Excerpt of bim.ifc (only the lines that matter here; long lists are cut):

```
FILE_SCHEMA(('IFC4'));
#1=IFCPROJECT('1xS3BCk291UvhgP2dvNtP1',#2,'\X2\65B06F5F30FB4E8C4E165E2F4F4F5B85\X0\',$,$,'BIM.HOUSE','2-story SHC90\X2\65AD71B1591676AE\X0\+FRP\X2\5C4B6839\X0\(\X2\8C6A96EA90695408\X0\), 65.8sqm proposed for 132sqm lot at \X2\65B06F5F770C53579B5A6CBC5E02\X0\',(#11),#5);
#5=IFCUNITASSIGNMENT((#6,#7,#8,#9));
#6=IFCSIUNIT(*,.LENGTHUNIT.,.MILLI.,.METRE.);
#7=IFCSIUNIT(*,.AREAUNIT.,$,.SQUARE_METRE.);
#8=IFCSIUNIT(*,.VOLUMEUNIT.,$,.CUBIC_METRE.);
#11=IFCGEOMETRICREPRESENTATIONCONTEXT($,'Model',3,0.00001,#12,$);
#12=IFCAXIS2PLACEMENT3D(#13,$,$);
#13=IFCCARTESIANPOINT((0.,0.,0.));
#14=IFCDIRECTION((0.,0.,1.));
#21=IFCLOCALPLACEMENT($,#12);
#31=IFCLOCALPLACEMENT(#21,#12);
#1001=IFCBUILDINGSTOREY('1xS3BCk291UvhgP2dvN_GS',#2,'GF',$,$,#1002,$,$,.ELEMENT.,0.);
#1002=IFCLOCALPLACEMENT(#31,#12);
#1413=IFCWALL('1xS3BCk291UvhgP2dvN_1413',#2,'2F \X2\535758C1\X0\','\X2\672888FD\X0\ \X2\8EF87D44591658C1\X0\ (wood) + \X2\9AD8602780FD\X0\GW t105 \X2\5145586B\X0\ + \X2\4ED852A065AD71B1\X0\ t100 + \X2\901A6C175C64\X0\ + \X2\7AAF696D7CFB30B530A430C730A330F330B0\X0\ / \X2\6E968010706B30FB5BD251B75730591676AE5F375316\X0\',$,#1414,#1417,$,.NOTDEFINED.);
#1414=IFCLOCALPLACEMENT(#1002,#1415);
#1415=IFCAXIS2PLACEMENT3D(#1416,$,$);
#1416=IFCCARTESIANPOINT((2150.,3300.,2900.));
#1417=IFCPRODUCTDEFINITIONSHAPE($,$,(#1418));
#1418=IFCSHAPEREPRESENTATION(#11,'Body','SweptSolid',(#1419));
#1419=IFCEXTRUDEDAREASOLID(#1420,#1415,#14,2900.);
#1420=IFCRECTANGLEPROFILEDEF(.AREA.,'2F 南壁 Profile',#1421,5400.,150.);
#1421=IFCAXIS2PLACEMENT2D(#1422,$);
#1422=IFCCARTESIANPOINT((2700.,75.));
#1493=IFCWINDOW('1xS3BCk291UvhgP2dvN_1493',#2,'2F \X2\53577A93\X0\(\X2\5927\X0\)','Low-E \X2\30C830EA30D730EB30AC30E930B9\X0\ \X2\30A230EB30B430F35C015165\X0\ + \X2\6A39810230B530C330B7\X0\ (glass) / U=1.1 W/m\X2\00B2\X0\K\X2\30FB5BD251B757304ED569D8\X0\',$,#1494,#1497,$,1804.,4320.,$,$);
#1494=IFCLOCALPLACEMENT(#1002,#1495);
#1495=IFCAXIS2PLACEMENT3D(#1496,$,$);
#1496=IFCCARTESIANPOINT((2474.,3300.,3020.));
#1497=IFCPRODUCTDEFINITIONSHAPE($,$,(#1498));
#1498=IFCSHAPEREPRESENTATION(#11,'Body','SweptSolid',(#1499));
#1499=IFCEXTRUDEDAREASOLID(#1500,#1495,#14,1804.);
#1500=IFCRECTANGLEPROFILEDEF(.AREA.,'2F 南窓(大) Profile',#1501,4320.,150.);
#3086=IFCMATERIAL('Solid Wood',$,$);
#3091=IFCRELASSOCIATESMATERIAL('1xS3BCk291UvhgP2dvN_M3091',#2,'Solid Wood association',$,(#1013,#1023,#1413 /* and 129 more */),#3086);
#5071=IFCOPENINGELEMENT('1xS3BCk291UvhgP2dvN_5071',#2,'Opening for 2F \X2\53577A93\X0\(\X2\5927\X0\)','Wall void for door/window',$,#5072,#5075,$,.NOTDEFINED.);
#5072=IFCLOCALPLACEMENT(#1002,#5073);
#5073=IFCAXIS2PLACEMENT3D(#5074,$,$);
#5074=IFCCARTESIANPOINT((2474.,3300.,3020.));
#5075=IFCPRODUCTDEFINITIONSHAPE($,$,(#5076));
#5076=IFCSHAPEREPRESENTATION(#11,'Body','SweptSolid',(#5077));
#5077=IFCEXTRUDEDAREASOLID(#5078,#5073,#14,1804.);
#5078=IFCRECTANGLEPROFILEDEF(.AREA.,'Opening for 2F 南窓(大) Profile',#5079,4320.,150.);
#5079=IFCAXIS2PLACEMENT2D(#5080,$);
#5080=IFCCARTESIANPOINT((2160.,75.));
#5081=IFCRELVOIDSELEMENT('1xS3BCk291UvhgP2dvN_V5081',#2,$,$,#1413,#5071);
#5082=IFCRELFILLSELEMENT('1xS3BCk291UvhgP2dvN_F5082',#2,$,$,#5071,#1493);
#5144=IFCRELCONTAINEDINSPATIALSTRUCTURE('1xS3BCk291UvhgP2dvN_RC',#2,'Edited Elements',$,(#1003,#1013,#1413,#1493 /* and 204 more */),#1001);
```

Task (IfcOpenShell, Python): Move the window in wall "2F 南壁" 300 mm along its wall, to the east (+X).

```python
import ifcopenshell
import ifcopenshell.api.geometry
import ifcopenshell.util.placement
import ifcopenshell.util.unit

model = ifcopenshell.open("bim.ifc")
unit_scale = ifcopenshell.util.unit.calculate_unit_scale(model)

window = model.by_guid("1xS3BCk291UvhgP2dvN_1493")
opening = window.FillsVoids[0].RelatingOpeningElement
wall = opening.VoidsElements[0].RelatingBuildingElement

wall_matrix = ifcopenshell.util.placement.get_local_placement(wall.ObjectPlacement)
shift = wall_matrix[:3, 0] * 0.3 / unit_scale
before = ifcopenshell.util.placement.get_local_placement(window.ObjectPlacement)[:3, 3].copy()

# The window is not placed relative to its opening, so move both.
for product in (opening, window):
    matrix = ifcopenshell.util.placement.get_local_placement(product.ObjectPlacement)
    matrix[:3, 3] += shift
    ifcopenshell.api.geometry.edit_object_placement(model, product=product, matrix=matrix, is_si=False)

after = ifcopenshell.util.placement.get_local_placement(window.ObjectPlacement)[:3, 3]
print("window moved by", (after - before).round(3) + 0.0)

model.write("bim_v2.ifc")
```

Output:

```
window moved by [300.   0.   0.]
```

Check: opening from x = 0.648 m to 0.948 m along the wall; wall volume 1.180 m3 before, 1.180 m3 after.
